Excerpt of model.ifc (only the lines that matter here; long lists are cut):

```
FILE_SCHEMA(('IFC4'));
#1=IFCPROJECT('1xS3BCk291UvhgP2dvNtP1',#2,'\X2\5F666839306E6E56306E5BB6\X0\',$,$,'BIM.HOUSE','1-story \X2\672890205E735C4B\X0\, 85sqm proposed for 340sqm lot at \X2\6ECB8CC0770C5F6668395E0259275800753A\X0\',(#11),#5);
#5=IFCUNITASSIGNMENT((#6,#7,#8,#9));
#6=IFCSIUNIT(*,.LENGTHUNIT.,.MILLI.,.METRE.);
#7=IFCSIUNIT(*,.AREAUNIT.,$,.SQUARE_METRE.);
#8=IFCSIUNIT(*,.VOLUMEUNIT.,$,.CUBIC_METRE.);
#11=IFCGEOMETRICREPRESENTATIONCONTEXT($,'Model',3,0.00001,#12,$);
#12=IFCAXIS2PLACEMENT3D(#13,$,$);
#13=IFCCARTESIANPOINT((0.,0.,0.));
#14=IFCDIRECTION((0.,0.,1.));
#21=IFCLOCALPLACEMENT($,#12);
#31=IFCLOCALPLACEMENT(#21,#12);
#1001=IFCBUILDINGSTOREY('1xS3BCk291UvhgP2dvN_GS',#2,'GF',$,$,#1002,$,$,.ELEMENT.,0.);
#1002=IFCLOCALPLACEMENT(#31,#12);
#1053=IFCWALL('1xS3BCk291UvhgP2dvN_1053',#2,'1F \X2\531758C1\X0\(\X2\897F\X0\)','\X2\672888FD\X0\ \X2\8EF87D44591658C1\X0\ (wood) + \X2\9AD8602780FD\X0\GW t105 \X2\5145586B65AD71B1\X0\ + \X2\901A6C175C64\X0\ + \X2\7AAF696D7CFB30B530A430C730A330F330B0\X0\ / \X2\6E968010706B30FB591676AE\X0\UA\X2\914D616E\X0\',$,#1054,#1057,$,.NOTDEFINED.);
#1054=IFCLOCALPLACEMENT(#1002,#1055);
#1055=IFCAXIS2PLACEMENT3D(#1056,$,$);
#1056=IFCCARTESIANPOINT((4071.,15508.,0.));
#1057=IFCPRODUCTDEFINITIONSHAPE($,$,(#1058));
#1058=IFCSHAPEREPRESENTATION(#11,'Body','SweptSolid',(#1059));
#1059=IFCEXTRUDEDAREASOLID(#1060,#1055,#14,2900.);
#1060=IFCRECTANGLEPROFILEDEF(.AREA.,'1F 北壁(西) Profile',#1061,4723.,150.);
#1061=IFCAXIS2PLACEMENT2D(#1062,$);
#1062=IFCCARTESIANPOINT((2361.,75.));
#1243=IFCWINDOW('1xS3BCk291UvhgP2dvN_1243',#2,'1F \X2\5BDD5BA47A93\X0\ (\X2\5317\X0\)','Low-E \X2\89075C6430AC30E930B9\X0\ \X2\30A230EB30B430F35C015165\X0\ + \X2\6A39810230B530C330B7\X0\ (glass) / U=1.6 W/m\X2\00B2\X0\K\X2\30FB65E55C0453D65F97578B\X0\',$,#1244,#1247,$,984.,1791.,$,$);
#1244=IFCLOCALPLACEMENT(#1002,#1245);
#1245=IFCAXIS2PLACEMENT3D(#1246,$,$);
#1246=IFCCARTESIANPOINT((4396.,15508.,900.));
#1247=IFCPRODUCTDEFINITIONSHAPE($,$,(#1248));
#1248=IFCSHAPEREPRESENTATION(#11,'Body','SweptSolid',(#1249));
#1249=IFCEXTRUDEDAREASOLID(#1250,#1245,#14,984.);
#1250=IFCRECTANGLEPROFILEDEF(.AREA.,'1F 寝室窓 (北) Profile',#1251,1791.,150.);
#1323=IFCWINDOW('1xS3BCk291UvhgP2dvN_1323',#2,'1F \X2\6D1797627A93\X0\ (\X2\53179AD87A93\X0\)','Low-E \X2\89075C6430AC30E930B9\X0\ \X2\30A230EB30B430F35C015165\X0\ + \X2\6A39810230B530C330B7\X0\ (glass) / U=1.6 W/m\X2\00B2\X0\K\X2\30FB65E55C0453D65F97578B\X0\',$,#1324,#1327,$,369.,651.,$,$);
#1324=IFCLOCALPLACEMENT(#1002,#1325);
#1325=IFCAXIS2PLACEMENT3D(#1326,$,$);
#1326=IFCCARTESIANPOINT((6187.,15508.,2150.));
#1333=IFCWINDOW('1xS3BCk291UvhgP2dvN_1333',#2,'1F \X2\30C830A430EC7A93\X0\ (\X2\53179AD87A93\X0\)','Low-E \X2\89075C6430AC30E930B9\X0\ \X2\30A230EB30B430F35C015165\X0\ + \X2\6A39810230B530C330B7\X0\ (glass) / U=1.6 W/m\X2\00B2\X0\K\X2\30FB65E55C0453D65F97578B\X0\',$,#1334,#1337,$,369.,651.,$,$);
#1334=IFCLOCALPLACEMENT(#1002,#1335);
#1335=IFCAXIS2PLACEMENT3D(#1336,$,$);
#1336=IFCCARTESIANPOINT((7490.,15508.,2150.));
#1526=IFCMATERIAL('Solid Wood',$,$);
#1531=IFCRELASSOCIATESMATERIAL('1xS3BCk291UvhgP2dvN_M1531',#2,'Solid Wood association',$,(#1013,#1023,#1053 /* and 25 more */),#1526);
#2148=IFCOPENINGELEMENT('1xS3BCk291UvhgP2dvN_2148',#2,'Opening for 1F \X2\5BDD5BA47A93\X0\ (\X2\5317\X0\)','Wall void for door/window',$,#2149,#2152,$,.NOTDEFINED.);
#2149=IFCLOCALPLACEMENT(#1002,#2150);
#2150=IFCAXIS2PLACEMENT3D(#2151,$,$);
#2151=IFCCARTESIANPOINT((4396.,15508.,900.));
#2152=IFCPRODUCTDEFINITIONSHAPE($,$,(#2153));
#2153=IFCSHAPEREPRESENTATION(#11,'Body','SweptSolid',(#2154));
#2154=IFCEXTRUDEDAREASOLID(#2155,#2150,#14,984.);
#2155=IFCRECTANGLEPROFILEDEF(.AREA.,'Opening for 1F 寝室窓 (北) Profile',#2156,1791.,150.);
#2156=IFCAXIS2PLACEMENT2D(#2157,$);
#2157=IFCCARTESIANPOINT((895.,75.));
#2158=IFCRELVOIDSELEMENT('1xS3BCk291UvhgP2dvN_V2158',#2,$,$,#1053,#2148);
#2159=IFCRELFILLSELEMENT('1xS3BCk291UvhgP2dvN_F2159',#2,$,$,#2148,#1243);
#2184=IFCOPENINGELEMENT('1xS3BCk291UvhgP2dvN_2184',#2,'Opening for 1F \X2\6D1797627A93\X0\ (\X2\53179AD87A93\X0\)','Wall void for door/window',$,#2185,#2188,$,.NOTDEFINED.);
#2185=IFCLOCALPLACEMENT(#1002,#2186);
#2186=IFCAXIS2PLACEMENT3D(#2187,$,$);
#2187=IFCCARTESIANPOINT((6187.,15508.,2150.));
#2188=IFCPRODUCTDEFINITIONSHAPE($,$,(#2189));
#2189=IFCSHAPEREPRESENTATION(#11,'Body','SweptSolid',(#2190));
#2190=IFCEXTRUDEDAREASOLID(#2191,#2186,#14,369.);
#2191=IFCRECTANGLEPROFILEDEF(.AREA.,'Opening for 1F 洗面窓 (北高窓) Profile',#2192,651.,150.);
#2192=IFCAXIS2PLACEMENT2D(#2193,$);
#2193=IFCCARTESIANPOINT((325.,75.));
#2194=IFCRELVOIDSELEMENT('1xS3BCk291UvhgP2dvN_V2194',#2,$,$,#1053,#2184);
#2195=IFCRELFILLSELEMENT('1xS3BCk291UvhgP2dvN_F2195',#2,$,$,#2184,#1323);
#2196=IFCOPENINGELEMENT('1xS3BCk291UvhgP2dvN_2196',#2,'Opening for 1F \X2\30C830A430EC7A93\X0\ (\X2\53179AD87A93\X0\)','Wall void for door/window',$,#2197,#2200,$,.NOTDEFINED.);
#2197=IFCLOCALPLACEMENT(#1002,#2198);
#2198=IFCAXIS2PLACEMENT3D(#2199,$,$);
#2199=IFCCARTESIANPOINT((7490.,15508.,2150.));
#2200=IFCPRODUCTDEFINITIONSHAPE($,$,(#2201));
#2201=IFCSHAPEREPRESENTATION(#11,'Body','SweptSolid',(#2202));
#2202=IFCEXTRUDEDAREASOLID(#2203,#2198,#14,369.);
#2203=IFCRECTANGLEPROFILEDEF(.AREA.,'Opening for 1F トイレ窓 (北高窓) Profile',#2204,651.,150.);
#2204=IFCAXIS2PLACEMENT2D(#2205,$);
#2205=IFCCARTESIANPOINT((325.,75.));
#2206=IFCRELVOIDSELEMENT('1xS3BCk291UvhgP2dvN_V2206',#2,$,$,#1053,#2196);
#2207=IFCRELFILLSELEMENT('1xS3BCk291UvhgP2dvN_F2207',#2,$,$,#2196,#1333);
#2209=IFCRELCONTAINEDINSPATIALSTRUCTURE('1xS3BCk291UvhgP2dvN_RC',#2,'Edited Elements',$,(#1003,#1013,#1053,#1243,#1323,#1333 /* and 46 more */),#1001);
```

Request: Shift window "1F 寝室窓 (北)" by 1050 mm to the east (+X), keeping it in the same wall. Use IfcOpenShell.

```python
import ifcopenshell
import ifcopenshell.api.geometry
import ifcopenshell.util.placement
import ifcopenshell.util.unit

model = ifcopenshell.open("model.ifc")
unit_scale = ifcopenshell.util.unit.calculate_unit_scale(model)

window = model.by_guid("1xS3BCk291UvhgP2dvN_1243")
opening = window.FillsVoids[0].RelatingOpeningElement
wall = opening.VoidsElements[0].RelatingBuildingElement

wall_matrix = ifcopenshell.util.placement.get_local_placement(wall.ObjectPlacement)
shift = wall_matrix[:3, 0] * 1.05 / unit_scale
before = ifcopenshell.util.placement.get_local_placement(window.ObjectPlacement)[:3, 3].copy()

# The window is not placed relative to its opening, so move both.
for product in (opening, window):
    matrix = ifcopenshell.util.placement.get_local_placement(product.ObjectPlacement)
    matrix[:3, 3] += shift
    ifcopenshell.api.geometry.edit_object_placement(model, product=product, matrix=matrix, is_si=False)

after = ifcopenshell.util.placement.get_local_placement(window.ObjectPlacement)[:3, 3]
print("window moved by", (after - before).round(3) + 0.0)

model.write("model_edited.ifc")
```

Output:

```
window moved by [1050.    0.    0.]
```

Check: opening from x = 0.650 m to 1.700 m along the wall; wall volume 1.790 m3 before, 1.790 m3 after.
